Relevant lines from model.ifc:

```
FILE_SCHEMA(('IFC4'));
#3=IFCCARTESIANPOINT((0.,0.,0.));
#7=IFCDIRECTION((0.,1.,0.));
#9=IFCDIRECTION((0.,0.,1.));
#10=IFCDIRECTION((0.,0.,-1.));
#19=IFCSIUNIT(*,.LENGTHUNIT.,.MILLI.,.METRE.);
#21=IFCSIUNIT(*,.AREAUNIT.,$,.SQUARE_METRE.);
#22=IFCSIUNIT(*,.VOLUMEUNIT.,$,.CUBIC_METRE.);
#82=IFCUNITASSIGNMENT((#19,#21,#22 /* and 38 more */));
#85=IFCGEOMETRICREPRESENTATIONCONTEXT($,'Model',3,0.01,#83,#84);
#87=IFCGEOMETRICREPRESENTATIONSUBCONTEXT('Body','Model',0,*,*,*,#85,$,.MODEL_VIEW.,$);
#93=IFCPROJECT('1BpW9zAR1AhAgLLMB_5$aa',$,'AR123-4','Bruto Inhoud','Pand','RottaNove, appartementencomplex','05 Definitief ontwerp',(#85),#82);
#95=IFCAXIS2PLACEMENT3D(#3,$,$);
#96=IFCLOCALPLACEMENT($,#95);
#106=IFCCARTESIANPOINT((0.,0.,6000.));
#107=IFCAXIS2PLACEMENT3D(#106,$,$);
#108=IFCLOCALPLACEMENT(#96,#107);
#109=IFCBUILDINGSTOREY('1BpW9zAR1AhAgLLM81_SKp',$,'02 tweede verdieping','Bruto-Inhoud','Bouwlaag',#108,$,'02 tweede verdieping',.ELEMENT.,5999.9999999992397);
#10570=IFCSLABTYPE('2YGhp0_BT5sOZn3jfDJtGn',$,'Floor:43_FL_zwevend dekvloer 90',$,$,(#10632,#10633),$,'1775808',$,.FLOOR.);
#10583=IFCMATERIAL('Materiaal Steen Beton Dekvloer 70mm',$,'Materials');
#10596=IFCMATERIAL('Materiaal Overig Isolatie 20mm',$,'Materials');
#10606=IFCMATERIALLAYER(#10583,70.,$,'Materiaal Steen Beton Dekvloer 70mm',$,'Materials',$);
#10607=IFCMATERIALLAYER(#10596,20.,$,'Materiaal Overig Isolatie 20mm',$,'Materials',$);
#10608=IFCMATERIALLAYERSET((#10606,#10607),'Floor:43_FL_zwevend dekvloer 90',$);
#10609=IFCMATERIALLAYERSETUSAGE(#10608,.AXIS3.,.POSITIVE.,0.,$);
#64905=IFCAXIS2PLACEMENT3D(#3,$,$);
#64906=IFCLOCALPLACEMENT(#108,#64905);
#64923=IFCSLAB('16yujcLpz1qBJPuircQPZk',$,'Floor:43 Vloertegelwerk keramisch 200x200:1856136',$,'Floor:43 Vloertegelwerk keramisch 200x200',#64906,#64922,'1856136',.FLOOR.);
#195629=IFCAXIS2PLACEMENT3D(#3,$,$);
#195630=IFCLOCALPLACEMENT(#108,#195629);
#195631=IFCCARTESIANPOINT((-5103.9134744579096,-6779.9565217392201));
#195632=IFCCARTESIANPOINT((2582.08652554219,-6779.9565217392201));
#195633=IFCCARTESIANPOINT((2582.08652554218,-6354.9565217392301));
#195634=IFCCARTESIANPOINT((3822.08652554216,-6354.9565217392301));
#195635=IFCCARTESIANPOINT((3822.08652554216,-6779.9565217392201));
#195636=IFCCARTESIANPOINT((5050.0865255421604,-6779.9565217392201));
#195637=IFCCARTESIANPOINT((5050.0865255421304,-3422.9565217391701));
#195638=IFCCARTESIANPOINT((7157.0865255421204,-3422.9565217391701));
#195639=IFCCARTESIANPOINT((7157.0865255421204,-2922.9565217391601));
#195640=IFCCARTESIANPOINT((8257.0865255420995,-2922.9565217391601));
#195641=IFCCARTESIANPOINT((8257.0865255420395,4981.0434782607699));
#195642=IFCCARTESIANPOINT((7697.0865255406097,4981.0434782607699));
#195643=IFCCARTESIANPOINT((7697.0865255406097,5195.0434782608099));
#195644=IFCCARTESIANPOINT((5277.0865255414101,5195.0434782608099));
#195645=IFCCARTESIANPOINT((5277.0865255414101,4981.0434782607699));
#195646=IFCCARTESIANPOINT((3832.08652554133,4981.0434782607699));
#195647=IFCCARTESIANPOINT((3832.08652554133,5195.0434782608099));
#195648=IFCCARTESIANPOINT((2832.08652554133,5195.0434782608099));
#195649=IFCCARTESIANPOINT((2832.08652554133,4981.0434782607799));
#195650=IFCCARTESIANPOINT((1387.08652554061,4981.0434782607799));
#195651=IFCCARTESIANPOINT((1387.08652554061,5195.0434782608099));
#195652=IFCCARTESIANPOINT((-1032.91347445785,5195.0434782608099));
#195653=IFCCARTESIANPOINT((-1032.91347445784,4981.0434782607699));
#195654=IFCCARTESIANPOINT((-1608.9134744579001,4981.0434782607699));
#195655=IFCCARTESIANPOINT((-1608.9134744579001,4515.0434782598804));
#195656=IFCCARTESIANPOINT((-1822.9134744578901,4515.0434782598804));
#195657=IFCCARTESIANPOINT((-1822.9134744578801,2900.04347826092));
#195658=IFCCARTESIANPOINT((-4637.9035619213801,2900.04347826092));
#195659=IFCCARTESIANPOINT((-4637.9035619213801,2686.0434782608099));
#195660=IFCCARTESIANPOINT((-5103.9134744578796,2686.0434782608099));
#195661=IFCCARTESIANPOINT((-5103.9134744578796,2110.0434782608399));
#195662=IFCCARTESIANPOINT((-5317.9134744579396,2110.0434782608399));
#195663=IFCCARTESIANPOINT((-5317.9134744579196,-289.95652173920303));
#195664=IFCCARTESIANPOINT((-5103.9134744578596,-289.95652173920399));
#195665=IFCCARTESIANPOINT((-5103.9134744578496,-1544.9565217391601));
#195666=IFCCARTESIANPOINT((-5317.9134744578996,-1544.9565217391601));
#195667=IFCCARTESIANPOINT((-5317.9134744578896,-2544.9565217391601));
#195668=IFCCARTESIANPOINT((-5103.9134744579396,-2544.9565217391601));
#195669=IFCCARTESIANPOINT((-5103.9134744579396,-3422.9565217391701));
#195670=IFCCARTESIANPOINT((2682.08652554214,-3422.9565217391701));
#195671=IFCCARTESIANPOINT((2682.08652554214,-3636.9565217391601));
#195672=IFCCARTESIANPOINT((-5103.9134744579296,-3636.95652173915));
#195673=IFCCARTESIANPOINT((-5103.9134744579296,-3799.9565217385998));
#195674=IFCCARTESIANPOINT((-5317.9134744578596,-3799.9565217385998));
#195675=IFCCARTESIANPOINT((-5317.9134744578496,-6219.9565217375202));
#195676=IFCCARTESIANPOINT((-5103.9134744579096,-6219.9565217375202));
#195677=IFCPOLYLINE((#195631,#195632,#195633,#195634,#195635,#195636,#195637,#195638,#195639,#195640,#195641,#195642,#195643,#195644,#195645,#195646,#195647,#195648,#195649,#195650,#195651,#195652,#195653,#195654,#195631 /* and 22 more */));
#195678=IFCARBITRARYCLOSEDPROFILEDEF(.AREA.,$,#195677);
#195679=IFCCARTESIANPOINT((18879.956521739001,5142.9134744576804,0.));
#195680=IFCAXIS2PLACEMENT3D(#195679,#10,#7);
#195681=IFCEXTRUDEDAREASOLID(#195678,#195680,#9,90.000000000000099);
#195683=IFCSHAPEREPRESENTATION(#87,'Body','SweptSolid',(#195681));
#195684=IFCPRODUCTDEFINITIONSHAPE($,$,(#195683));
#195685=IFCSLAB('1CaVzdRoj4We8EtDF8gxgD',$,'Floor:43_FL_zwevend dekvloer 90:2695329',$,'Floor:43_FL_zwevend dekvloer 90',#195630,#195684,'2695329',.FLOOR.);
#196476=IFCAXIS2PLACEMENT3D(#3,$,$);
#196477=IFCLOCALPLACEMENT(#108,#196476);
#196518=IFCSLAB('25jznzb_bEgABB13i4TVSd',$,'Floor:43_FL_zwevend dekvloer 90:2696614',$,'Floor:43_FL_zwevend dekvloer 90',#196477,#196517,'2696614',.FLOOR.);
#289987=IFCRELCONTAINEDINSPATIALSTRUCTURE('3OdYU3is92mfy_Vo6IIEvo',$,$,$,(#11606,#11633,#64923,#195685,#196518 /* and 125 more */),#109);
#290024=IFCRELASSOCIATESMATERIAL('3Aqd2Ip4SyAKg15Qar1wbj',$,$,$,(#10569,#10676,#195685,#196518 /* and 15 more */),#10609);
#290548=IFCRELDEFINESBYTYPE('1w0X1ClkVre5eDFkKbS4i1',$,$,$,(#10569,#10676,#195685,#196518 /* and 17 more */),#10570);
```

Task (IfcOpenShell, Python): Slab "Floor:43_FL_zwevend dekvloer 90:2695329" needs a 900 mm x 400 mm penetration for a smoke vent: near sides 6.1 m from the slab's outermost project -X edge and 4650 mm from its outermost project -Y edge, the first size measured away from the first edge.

```python
import numpy as np
import ifcopenshell
import ifcopenshell.api.feature
import ifcopenshell.api.geometry
import ifcopenshell.api.root
import ifcopenshell.geom
import ifcopenshell.util.placement
import ifcopenshell.util.representation
import ifcopenshell.util.shape
import ifcopenshell.util.unit

model = ifcopenshell.open("model.ifc")
unit_scale = ifcopenshell.util.unit.calculate_unit_scale(model)
settings = ifcopenshell.geom.settings()


def volume(element):
    """Net volume in cubic metres, openings subtracted."""
    shape = ifcopenshell.geom.create_shape(settings, element)
    return ifcopenshell.util.shape.get_volume(shape.geometry)


slab = model.by_id(195685)
before = volume(slab)

# Extent in the slab's own axes, in metres. The edges named are its -X and -Y sides.
slab_shape = ifcopenshell.geom.create_shape(settings, slab)
vertices = ifcopenshell.util.shape.get_vertices(slab_shape.geometry)
x_min, y_min, bottom = vertices.min(axis=0)
top = vertices[:, 2].max()

opening = ifcopenshell.api.root.create_entity(model, ifc_class="IfcOpeningElement", name="Smoke vent opening", predefined_type="OPENING")
context = ifcopenshell.util.representation.get_context(model, "Model", "Body", "MODEL_VIEW")
width, depth = 0.9, 0.4
outline = [(0.0, 0.0), (width, 0.0), (width, depth), (0.0, depth), (0.0, 0.0)]
# Overshoot both faces by 50 mm so the cut is clean.
shape = ifcopenshell.api.geometry.add_slab_representation(
    model, context=context, depth=top - bottom + 0.1, polyline=outline
)
ifcopenshell.api.geometry.assign_representation(model, product=opening, representation=shape)

matrix = ifcopenshell.util.placement.get_local_placement(slab.ObjectPlacement)
matrix[:, 3] = matrix @ np.append(np.array([x_min + 6.1, y_min + 4.65, bottom - 0.05]) / unit_scale, 1.0)
ifcopenshell.api.geometry.edit_object_placement(model, product=opening, matrix=matrix, is_si=False)
ifcopenshell.api.feature.add_feature(model, feature=opening, element=slab)

after = volume(slab)

print(f"slab volume {before:.3f} -> {after:.3f} m3")

model.write("model_v2.ifc")
```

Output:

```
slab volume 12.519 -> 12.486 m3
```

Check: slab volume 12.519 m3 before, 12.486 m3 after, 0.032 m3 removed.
